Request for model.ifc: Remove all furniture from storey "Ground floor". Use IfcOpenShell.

First a look at what the model holds.

```python
import ifcopenshell
import ifcopenshell.util.element

model = ifcopenshell.open("model.ifc")
print(model.schema)
storey = next(s for s in model.by_type("IfcBuildingStorey") if s.Name == "Ground floor")
furniture = [e for e in ifcopenshell.util.element.get_decomposition(storey) if e.is_a("IfcFurnishingElement")]
seen = {}
for e in furniture:
    element_type = ifcopenshell.util.element.get_type(e)
    name = element_type.Name if element_type not in (None, e) else None
    seen[name] = seen.get(name, 0) + 1
for name, count in sorted(seen.items(), key=str):
    print(count, "x", name)
```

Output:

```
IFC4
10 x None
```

```python
import ifcopenshell
import ifcopenshell.api.root
import ifcopenshell.util.element

model = ifcopenshell.open("model.ifc")

storey = next(s for s in model.by_type("IfcBuildingStorey") if s.Name == "Ground floor")
furniture = [e for e in ifcopenshell.util.element.get_decomposition(storey) if e.is_a("IfcFurnishingElement")]

for e in furniture:
    ifcopenshell.api.root.remove_product(model, product=e)
print(len(furniture), "removed")

model.write("model_v2.ifc")
```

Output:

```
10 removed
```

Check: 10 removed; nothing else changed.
